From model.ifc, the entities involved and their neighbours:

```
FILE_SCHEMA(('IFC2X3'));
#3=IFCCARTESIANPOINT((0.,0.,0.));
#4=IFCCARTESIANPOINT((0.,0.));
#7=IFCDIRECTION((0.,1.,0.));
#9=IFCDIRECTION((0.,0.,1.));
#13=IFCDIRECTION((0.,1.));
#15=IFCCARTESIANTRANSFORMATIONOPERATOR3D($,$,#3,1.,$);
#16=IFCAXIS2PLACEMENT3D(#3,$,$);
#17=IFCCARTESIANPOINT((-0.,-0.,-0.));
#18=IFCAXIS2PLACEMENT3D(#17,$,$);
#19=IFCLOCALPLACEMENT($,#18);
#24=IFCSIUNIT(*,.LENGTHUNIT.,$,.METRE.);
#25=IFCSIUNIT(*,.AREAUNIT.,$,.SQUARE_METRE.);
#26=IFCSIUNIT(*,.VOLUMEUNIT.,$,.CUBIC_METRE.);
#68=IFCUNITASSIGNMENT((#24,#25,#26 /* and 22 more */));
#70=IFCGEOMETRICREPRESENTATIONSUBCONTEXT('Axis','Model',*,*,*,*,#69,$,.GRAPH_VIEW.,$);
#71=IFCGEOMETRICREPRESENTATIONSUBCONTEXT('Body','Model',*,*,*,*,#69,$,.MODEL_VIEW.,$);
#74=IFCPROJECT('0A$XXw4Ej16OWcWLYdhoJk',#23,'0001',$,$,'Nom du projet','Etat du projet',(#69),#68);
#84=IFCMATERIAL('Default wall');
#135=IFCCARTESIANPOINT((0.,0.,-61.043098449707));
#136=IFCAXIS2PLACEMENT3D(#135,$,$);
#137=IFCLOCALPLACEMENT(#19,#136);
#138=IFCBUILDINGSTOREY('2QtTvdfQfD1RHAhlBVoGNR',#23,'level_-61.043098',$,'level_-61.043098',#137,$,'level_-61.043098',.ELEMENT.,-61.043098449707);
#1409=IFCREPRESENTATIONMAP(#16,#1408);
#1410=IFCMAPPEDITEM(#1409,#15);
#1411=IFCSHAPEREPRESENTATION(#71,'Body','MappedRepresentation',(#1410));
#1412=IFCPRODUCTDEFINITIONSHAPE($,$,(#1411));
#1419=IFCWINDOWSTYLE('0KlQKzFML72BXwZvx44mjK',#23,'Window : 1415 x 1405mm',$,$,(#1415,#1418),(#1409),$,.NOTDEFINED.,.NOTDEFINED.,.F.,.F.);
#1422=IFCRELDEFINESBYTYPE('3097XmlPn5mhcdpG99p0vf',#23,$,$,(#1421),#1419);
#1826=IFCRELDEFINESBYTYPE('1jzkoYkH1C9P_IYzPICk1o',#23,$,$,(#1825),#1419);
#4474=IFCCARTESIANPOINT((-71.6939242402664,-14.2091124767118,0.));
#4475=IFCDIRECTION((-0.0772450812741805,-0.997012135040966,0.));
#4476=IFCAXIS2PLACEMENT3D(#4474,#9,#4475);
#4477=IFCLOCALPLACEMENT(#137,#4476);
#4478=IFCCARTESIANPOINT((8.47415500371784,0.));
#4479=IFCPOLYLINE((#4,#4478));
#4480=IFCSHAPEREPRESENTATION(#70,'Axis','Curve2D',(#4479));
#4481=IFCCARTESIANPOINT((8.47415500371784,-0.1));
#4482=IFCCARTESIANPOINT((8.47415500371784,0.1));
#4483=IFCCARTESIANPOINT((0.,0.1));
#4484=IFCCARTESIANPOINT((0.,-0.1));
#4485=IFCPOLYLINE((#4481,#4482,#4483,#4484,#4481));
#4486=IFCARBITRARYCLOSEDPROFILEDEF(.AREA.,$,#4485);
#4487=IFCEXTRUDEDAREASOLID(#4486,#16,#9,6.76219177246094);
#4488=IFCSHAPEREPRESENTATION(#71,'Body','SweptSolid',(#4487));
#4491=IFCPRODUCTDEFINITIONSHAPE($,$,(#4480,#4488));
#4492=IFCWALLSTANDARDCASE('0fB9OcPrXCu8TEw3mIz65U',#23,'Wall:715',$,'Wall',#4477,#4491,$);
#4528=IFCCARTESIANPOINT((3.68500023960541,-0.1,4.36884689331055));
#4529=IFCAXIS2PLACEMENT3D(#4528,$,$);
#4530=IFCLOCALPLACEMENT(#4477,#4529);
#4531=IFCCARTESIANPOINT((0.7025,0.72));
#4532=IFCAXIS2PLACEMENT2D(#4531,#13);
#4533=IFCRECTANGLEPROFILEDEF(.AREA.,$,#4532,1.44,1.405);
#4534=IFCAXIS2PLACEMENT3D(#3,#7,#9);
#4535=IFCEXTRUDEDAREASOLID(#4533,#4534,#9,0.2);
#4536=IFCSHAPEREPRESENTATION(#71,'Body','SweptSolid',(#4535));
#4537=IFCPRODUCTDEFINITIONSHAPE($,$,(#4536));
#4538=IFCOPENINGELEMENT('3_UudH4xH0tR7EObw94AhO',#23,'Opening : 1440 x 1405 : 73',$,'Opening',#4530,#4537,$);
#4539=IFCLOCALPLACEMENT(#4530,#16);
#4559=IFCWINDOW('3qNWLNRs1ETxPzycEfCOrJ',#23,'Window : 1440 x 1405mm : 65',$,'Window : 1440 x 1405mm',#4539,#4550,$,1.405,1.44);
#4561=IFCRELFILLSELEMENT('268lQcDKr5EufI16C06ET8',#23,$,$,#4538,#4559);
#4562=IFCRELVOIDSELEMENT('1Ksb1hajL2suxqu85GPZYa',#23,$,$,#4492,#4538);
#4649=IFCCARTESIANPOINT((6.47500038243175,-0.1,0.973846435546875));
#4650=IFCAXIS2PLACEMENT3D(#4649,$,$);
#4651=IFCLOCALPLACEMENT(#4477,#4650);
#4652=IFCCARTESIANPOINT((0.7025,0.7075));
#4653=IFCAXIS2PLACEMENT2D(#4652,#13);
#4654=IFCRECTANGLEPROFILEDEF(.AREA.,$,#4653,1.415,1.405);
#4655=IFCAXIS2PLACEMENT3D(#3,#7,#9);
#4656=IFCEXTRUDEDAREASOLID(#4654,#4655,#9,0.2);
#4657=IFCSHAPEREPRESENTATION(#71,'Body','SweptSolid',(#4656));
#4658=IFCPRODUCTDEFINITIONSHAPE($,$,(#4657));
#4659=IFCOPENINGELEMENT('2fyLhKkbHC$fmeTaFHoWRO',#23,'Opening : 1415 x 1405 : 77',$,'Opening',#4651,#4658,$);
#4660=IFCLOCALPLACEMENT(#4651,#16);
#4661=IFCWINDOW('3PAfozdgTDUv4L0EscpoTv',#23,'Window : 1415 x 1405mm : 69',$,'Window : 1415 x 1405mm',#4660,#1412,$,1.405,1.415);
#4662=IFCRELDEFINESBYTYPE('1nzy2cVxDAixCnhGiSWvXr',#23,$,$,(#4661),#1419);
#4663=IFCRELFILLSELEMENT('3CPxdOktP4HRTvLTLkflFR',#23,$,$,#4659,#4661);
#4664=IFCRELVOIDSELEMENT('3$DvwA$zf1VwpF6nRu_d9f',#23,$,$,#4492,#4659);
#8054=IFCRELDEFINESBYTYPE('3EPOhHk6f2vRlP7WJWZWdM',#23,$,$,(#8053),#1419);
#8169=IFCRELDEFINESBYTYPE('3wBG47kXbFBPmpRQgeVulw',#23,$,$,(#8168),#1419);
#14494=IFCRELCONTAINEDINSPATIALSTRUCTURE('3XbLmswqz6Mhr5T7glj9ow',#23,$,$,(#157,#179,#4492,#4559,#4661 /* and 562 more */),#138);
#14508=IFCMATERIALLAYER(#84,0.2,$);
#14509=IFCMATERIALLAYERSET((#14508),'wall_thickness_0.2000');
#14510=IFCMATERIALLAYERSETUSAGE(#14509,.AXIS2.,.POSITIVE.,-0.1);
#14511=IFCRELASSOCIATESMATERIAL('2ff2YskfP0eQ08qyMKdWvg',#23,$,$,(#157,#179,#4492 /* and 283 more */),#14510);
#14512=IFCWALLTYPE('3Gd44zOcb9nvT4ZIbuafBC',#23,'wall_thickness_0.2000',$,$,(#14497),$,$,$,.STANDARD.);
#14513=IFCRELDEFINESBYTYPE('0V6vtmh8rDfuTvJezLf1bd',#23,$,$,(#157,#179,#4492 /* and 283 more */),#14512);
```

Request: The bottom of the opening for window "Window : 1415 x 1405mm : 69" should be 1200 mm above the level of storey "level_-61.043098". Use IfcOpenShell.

```python
import numpy as np
import ifcopenshell
import ifcopenshell.api.geometry
import ifcopenshell.geom
import ifcopenshell.util.element
import ifcopenshell.util.placement
import ifcopenshell.util.shape
import ifcopenshell.util.unit

model = ifcopenshell.open("model.ifc")
unit_scale = ifcopenshell.util.unit.calculate_unit_scale(model)

window = model.by_guid("3PAfozdgTDUv4L0EscpoTv")
opening = window.FillsVoids[0].RelatingOpeningElement
storey = ifcopenshell.util.element.get_container(window, ifc_class="IfcBuildingStorey")
level = ifcopenshell.util.placement.get_local_placement(storey.ObjectPlacement)[2, 3]

# The opening's origin need not be at the sill, so measure its lowest point.
shape = ifcopenshell.geom.create_shape(ifcopenshell.geom.settings(), opening)
bottom = ifcopenshell.util.shape.get_shape_bottom_elevation(shape, shape.geometry) / unit_scale
dz = level + 1.2 / unit_scale - bottom

shift = np.array([0.0, 0.0, dz])
# The window is placed relative to its opening, so it follows when the opening moves.
matrix = ifcopenshell.util.placement.get_local_placement(opening.ObjectPlacement)
matrix[:3, 3] += shift
ifcopenshell.api.geometry.edit_object_placement(
    model, product=opening, matrix=matrix, is_si=False, should_transform_children=True
)

print(f"moved by {dz * unit_scale:+.3f} m")

model.write("model_v2.ifc")
```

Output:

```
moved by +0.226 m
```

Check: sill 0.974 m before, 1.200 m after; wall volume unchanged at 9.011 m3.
